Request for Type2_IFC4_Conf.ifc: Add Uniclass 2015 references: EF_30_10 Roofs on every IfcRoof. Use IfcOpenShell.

First a look at what the model holds.

```python
import ifcopenshell

model = ifcopenshell.open("Type2_IFC4_Conf.ifc")
print(model.schema)
print("classifications:", [c.Name for c in model.by_type("IfcClassification")])
for ifc_class in ("IfcDoor", "IfcRoof", "IfcStair", "IfcWall", "IfcWindow"):
    print(ifc_class, len(model.by_type(ifc_class)))
```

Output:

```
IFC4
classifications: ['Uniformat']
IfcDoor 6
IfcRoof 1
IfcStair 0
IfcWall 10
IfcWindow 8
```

```python
import ifcopenshell
import ifcopenshell.api.classification

model = ifcopenshell.open("Type2_IFC4_Conf.ifc")

system = ifcopenshell.api.classification.add_classification(model, classification="Uniclass 2015")

codes = {
    "IfcRoof": ("EF_30_10", "Roofs"),
}
for ifc_class, (code, name) in codes.items():
    products = model.by_type(ifc_class)
    ifcopenshell.api.classification.add_reference(
        model, products=products, classification=system, identification=code, name=name
    )
    print(code, len(products))

model.write("Type2_IFC4_Conf_rev.ifc")
```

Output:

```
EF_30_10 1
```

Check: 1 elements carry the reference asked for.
